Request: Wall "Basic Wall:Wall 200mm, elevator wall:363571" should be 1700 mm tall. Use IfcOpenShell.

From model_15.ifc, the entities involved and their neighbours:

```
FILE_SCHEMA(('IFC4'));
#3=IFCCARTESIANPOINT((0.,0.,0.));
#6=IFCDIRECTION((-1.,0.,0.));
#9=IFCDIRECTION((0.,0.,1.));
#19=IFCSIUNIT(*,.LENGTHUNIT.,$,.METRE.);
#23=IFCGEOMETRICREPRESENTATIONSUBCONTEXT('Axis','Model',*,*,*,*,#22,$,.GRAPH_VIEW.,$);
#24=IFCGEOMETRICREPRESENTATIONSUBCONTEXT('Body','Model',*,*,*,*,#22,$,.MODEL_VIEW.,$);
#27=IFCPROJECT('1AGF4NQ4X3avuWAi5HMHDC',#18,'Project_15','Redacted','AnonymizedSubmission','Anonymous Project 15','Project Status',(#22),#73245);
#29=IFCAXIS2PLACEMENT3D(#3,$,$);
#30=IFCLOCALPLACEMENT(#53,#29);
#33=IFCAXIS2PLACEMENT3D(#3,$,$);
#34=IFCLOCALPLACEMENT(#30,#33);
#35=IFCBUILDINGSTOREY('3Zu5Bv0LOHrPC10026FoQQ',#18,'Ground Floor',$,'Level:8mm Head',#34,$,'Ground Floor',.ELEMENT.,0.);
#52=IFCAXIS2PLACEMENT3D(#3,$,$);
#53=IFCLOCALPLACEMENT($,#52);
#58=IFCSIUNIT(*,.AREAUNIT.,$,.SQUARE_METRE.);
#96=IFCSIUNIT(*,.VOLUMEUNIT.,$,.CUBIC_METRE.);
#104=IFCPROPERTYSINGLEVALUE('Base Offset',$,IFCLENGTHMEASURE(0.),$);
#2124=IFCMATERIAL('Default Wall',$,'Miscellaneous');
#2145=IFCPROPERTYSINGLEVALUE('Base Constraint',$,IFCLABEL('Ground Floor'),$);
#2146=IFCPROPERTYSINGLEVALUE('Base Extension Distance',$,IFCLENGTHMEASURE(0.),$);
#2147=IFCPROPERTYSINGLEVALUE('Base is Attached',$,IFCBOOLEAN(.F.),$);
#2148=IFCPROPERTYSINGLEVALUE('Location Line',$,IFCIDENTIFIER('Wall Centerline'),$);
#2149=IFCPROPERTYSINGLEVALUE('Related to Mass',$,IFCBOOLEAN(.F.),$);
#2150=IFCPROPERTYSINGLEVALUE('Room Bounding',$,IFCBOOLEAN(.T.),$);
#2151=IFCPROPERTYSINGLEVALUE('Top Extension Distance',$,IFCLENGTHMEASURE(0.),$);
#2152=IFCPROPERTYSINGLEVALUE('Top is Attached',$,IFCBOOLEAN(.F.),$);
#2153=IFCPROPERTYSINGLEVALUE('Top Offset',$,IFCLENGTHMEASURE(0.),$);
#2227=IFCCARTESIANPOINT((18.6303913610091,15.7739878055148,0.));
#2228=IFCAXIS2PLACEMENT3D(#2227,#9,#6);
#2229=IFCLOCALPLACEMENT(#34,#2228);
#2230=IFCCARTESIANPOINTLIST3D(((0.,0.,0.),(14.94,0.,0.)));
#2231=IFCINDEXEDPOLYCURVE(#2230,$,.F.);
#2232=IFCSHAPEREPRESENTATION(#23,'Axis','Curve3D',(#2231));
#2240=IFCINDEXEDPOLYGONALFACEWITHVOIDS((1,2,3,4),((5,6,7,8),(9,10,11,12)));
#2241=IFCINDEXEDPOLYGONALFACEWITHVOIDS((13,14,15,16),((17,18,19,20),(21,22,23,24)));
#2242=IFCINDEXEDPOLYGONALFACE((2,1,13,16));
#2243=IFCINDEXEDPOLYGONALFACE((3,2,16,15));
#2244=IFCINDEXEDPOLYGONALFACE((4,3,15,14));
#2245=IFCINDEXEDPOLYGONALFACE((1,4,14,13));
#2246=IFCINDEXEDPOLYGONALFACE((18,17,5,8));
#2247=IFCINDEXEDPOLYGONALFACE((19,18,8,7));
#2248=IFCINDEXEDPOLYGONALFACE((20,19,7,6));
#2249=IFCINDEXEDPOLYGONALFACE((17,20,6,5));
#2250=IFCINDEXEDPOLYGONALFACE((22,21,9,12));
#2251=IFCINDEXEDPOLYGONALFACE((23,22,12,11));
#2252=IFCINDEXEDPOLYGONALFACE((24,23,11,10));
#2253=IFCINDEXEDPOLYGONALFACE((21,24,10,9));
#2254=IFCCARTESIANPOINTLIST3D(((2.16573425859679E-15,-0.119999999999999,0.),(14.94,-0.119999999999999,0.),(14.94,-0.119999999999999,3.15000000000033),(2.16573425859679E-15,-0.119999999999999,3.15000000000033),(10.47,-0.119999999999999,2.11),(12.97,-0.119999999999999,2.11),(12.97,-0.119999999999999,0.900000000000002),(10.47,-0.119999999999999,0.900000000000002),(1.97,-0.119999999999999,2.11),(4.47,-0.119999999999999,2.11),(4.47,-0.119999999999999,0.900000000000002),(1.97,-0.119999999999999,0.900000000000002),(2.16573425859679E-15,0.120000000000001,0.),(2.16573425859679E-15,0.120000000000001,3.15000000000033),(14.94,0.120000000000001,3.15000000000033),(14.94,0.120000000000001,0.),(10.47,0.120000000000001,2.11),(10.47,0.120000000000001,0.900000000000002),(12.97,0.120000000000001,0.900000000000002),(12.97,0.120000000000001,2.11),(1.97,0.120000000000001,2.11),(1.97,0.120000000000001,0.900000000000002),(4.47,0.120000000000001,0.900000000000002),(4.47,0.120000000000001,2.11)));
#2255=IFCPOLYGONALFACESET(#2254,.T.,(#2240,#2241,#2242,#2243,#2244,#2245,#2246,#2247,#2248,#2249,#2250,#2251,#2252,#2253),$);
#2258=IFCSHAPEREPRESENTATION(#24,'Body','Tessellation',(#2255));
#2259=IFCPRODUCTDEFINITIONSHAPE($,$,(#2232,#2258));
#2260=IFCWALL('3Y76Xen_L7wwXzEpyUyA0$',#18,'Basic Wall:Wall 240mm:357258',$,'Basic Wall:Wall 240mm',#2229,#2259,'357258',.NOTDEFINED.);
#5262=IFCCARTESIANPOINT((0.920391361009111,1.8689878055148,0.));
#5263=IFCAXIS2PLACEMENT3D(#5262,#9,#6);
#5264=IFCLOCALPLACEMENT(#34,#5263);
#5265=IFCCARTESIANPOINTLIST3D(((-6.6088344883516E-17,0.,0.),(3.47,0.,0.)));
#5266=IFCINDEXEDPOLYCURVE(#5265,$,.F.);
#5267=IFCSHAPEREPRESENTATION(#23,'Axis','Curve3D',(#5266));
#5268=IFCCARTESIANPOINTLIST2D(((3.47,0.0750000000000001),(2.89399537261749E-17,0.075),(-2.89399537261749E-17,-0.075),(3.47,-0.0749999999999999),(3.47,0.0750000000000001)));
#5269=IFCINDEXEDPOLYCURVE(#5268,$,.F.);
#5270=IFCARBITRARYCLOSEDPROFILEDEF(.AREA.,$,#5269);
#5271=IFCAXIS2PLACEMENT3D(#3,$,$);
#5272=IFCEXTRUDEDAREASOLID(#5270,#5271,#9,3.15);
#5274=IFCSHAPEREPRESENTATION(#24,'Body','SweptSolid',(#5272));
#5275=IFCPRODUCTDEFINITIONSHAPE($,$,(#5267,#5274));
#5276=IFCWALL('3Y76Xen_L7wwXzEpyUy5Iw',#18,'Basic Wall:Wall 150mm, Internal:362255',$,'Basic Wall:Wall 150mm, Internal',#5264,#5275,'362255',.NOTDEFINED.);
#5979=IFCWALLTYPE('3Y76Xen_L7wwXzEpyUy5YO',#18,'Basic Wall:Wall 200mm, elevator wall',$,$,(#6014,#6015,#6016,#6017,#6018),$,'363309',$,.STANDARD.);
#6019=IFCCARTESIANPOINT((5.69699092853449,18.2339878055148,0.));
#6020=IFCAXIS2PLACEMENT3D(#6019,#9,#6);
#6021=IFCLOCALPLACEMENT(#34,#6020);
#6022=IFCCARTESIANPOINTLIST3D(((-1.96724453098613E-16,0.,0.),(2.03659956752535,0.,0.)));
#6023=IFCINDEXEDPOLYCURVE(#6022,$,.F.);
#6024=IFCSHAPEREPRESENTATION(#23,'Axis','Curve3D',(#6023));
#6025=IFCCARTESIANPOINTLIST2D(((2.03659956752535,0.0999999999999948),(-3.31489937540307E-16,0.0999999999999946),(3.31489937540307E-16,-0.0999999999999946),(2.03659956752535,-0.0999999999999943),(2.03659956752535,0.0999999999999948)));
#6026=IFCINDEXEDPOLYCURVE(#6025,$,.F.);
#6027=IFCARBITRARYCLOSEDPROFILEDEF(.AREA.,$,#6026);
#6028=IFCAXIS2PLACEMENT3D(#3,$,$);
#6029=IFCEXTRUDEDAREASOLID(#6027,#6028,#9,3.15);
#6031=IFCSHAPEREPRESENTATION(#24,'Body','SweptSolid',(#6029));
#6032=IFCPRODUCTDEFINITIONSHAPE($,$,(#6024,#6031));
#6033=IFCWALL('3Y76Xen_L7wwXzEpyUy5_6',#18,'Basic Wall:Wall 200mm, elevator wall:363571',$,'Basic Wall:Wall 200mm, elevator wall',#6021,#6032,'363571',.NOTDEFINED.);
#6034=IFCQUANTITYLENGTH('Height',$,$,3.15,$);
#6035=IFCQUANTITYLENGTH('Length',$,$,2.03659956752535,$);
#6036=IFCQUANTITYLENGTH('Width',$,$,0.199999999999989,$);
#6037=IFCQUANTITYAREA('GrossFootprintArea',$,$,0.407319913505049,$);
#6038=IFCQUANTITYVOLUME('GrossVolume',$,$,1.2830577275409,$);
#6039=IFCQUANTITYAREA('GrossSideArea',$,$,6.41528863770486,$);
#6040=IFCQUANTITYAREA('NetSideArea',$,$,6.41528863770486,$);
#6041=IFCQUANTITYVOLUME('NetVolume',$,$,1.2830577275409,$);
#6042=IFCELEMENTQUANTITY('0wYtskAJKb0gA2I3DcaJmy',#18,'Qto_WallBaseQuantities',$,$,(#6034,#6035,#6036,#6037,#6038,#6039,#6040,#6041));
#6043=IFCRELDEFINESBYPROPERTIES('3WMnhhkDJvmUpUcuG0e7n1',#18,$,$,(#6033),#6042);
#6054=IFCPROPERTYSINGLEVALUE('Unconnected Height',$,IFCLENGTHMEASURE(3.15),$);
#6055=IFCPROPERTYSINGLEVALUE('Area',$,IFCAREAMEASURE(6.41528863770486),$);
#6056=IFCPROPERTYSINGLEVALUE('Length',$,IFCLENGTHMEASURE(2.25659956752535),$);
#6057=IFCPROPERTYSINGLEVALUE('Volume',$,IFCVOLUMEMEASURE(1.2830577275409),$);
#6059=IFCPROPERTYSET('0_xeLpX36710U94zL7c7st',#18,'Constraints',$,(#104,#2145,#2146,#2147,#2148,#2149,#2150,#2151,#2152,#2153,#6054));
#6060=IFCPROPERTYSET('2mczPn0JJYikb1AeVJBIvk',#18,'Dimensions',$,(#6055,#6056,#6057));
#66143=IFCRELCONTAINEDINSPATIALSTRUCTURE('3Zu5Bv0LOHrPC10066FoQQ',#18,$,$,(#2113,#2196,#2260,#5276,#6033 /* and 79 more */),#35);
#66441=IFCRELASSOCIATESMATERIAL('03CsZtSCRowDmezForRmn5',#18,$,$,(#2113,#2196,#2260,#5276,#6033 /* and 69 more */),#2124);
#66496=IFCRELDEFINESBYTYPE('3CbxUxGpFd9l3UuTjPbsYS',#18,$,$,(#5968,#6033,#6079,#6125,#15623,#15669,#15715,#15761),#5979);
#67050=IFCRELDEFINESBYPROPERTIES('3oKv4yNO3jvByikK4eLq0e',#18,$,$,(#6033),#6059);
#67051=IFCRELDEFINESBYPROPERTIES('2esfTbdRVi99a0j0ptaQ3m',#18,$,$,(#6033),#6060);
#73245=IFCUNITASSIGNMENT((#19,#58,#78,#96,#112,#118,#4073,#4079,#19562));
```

```python
import ifcopenshell
import ifcopenshell.api.pset
import ifcopenshell.geom
import ifcopenshell.util.element
import ifcopenshell.util.representation
import ifcopenshell.util.shape
import ifcopenshell.util.unit

model = ifcopenshell.open("model_15.ifc")
unit_scale = ifcopenshell.util.unit.calculate_unit_scale(model)
area_scale = ifcopenshell.util.unit.calculate_unit_scale(model, "AREAUNIT")
volume_scale = ifcopenshell.util.unit.calculate_unit_scale(model, "VOLUMEUNIT")
settings = ifcopenshell.geom.settings()


def volume(element):
    """Net volume in cubic metres, openings subtracted."""
    shape = ifcopenshell.geom.create_shape(settings, element)
    return ifcopenshell.util.shape.get_volume(shape.geometry)


wall = model.by_guid("3Y76Xen_L7wwXzEpyUy5_6")
before = volume(wall)

body = ifcopenshell.util.representation.get_representation(wall, "Model", "Body")
solid = body.Items[0]
old_height = solid.Depth
solid.Depth = 1.7 / unit_scale
after = volume(wall)
thickness = 0.2  # wall thickness in metres

# Update the stored height, areas and volumes.
qto = model.by_id(ifcopenshell.util.element.get_pset(wall, "Qto_WallBaseQuantities", should_inherit=False)["id"])
ifcopenshell.api.pset.edit_qto(model, qto=qto, properties={
    "Height": solid.Depth,
    "GrossVolume": ifcopenshell.util.element.get_pset(wall, "Qto_WallBaseQuantities", "GrossVolume") * solid.Depth / old_height,
    "GrossSideArea": ifcopenshell.util.element.get_pset(wall, "Qto_WallBaseQuantities", "GrossSideArea") * solid.Depth / old_height,
    "NetSideArea": after / thickness / area_scale,
    "NetVolume": after / volume_scale,
})
pset = model.by_id(ifcopenshell.util.element.get_pset(wall, "Constraints", should_inherit=False)["id"])
ifcopenshell.api.pset.edit_pset(model, pset=pset, properties={
    "Unconnected Height": model.create_entity("IfcLengthMeasure", solid.Depth),
})
pset = model.by_id(ifcopenshell.util.element.get_pset(wall, "Dimensions", should_inherit=False)["id"])
ifcopenshell.api.pset.edit_pset(model, pset=pset, properties={
    "Area": model.create_entity("IfcAreaMeasure", after / thickness / area_scale),
    "Volume": model.create_entity("IfcVolumeMeasure", after / volume_scale),
})

print(f"height {old_height:g} -> {solid.Depth:g}, volume {before:.3f} -> {after:.3f} m3")

model.write("model_15_updated.ifc")
```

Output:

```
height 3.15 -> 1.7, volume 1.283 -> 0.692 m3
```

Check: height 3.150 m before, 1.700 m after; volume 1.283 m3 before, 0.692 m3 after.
